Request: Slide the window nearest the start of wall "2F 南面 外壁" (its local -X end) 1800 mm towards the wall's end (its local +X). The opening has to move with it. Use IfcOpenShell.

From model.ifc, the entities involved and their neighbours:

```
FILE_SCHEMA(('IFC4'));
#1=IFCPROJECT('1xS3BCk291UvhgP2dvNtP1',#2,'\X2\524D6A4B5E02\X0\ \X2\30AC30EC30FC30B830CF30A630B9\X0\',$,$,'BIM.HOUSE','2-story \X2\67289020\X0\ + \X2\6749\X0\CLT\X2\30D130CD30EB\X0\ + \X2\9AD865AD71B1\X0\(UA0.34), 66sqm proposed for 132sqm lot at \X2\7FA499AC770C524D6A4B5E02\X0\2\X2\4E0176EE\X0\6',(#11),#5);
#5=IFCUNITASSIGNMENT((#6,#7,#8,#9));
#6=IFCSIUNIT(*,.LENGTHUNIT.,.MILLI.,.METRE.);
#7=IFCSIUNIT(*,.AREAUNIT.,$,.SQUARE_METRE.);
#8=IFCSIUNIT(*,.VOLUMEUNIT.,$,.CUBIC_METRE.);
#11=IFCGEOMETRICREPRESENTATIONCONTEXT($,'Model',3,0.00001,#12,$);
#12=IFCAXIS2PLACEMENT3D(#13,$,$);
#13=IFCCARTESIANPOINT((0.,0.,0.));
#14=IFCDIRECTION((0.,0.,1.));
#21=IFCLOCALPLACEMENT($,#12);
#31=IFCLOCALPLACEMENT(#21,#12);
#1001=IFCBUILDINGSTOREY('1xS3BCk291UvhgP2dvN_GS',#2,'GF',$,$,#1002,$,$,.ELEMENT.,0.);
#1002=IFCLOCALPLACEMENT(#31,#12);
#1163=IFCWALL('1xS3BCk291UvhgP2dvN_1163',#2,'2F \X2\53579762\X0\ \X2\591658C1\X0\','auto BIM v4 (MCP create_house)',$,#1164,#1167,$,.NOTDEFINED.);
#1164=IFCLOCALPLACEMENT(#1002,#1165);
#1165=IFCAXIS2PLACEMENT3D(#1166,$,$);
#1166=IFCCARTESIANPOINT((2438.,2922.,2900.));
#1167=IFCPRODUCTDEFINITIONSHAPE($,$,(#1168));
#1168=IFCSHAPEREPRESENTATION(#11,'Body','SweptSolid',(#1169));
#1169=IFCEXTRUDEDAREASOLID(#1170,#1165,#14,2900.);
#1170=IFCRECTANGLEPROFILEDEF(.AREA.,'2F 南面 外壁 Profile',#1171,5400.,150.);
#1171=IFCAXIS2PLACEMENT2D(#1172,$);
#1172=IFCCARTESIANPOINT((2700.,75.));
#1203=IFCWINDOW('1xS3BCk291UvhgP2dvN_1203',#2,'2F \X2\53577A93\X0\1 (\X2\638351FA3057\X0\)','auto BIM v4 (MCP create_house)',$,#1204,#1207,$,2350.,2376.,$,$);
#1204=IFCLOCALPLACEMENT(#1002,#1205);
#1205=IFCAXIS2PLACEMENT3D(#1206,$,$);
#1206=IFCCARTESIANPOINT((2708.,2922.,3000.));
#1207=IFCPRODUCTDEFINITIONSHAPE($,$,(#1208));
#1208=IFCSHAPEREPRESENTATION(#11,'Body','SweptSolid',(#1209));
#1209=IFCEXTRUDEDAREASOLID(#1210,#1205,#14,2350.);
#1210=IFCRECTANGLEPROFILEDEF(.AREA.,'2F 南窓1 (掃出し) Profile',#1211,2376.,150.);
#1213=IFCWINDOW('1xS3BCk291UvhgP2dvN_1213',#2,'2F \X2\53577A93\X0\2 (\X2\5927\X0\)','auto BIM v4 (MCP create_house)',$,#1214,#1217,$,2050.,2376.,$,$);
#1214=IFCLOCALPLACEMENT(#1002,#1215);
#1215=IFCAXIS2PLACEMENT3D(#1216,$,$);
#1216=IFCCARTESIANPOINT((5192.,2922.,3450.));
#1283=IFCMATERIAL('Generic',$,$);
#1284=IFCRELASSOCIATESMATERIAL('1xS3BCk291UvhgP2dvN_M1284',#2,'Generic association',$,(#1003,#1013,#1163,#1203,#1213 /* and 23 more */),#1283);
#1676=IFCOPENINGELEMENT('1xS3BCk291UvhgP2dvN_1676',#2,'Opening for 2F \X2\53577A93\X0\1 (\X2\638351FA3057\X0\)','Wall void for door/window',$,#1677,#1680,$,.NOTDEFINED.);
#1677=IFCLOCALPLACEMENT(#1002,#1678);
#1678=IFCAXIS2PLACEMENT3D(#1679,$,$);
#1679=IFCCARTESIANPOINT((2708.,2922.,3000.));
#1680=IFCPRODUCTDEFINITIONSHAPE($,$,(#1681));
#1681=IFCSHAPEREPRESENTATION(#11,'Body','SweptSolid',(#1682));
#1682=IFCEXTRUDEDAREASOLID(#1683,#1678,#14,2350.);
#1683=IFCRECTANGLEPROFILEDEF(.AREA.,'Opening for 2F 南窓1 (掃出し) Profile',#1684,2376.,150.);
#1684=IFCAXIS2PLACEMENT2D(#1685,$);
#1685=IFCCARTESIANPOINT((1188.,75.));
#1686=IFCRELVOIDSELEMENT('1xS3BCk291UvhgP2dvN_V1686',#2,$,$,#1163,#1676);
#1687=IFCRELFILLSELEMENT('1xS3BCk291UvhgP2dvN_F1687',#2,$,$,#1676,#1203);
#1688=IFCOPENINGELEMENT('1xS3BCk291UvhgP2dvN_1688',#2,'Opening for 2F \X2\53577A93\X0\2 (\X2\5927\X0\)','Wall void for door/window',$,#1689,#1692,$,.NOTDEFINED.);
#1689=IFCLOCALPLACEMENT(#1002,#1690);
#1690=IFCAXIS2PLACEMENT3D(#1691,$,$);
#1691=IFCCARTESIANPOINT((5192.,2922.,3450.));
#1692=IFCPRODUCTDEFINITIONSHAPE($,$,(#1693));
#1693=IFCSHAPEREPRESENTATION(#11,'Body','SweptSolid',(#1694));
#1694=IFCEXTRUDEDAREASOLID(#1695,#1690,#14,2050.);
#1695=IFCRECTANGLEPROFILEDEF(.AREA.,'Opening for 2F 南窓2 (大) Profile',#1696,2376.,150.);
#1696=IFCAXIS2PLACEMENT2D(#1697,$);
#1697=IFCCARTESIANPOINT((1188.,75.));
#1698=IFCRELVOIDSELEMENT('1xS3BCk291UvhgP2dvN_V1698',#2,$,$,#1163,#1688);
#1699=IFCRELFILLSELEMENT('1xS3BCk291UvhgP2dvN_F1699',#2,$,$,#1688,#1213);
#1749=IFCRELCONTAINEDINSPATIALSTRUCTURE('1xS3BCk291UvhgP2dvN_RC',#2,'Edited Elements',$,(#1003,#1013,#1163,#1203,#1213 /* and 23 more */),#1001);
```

```python
import ifcopenshell
import ifcopenshell.api.geometry
import ifcopenshell.util.placement

model = ifcopenshell.open("model.ifc")

window = model.by_id(1203)
opening = window.FillsVoids[0].RelatingOpeningElement
wall = opening.VoidsElements[0].RelatingBuildingElement

wall_matrix = ifcopenshell.util.placement.get_local_placement(wall.ObjectPlacement)
shift = wall_matrix[:3, 0] * 1800.0
before = ifcopenshell.util.placement.get_local_placement(window.ObjectPlacement)[:3, 3].copy()

# The window is not placed relative to its opening, so move both.
for product in (opening, window):
    matrix = ifcopenshell.util.placement.get_local_placement(product.ObjectPlacement)
    matrix[:3, 3] += shift
    ifcopenshell.api.geometry.edit_object_placement(model, product=product, matrix=matrix, is_si=False)

after = ifcopenshell.util.placement.get_local_placement(window.ObjectPlacement)[:3, 3]
print("window moved by", (after - before).round(3) + 0.0)

model.write("model-out.ifc")
```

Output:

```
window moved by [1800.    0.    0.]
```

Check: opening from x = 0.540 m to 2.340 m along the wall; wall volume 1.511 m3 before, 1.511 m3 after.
